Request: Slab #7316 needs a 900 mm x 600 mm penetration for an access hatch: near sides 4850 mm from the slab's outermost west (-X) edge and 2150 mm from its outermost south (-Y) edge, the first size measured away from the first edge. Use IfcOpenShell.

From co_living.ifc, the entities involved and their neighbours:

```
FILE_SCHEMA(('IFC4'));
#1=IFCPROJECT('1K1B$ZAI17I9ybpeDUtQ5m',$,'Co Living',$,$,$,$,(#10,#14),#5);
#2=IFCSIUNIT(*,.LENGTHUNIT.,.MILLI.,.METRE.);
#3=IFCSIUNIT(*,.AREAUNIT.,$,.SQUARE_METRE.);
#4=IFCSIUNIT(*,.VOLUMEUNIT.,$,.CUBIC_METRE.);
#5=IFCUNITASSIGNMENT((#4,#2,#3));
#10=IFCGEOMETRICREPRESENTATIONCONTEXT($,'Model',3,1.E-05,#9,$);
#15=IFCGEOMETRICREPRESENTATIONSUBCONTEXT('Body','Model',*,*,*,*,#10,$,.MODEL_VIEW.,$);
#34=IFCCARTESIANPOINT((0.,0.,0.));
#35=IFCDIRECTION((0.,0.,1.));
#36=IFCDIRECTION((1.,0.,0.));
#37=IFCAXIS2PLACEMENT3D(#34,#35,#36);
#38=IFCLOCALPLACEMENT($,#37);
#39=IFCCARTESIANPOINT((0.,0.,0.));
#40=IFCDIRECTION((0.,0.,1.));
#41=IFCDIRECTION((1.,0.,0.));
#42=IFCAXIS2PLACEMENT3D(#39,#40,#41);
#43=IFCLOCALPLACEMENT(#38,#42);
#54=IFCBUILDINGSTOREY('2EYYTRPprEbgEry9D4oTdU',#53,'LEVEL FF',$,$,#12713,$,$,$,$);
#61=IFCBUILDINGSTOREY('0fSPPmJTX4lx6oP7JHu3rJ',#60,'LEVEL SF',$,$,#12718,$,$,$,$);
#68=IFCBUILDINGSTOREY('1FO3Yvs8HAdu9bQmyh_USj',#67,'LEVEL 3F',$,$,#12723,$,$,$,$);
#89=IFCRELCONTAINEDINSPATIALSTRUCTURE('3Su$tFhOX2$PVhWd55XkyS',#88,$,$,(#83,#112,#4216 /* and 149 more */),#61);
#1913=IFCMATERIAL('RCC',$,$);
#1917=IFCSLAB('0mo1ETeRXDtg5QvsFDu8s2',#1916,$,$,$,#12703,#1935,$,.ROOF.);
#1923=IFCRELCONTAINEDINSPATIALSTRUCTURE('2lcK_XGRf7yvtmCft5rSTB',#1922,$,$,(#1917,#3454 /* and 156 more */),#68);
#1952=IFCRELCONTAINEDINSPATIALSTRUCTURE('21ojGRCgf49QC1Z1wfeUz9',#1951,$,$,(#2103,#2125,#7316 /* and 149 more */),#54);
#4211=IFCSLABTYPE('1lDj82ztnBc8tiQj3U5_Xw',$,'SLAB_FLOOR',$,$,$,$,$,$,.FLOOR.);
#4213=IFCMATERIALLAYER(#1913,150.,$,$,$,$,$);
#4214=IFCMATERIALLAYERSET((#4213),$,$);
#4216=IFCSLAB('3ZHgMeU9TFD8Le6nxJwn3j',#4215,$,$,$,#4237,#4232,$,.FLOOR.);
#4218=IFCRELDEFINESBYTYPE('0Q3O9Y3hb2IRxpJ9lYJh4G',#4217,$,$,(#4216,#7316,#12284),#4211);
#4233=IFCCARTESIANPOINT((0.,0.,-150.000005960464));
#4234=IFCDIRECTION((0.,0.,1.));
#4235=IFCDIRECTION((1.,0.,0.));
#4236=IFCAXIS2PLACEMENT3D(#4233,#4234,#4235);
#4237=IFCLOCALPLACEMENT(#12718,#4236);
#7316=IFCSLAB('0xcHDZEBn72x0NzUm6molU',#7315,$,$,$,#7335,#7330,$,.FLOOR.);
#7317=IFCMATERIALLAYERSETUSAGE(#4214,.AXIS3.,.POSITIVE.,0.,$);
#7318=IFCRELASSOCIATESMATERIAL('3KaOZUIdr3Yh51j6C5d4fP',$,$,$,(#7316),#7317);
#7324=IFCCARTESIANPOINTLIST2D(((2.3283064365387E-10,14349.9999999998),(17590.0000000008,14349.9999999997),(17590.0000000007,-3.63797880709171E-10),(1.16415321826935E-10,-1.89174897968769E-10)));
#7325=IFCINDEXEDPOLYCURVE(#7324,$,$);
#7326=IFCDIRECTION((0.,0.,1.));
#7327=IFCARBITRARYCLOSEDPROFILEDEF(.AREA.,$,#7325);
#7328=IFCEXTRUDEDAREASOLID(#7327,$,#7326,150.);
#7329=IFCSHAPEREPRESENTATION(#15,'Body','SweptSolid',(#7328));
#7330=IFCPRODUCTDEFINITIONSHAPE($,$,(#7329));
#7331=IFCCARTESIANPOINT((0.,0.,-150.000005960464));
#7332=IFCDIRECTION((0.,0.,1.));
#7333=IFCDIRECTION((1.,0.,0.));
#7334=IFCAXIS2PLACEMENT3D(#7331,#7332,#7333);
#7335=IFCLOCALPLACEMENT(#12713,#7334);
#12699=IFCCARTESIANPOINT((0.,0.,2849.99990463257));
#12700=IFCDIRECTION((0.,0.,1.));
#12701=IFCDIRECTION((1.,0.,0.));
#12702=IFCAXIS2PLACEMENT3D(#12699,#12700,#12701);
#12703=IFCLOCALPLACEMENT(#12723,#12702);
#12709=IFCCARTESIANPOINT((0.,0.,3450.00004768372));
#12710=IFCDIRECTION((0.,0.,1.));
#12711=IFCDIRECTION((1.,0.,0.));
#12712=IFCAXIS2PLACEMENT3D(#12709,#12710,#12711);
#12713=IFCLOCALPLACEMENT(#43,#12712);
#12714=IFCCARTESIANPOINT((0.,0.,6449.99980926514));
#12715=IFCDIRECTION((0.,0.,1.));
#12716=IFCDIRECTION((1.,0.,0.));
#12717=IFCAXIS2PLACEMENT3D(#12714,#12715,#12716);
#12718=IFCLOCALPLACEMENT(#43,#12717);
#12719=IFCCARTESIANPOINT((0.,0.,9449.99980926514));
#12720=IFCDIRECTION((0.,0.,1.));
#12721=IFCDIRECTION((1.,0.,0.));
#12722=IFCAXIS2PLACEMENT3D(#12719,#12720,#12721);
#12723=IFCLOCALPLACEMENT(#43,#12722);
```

```python
import numpy as np
import ifcopenshell
import ifcopenshell.api.feature
import ifcopenshell.api.geometry
import ifcopenshell.api.root
import ifcopenshell.geom
import ifcopenshell.util.placement
import ifcopenshell.util.representation
import ifcopenshell.util.shape
import ifcopenshell.util.unit

model = ifcopenshell.open("co_living.ifc")
unit_scale = ifcopenshell.util.unit.calculate_unit_scale(model)
settings = ifcopenshell.geom.settings()


def volume(element):
    """Net volume in cubic metres, openings subtracted."""
    shape = ifcopenshell.geom.create_shape(settings, element)
    return ifcopenshell.util.shape.get_volume(shape.geometry)


slab = model.by_id(7316)
before = volume(slab)

# Extent in the slab's own axes, in metres. The edges named are its -X and -Y sides.
slab_shape = ifcopenshell.geom.create_shape(settings, slab)
vertices = ifcopenshell.util.shape.get_vertices(slab_shape.geometry)
x_min, y_min, bottom = vertices.min(axis=0)
top = vertices[:, 2].max()

opening = ifcopenshell.api.root.create_entity(model, ifc_class="IfcOpeningElement", name="Access hatch opening", predefined_type="OPENING")
context = ifcopenshell.util.representation.get_context(model, "Model", "Body", "MODEL_VIEW")
width, depth = 0.9, 0.6
outline = [(0.0, 0.0), (width, 0.0), (width, depth), (0.0, depth), (0.0, 0.0)]
# Overshoot both faces by 50 mm so the cut is clean.
shape = ifcopenshell.api.geometry.add_slab_representation(
    model, context=context, depth=top - bottom + 0.1, polyline=outline
)
ifcopenshell.api.geometry.assign_representation(model, product=opening, representation=shape)

matrix = ifcopenshell.util.placement.get_local_placement(slab.ObjectPlacement)
matrix[:, 3] = matrix @ np.append(np.array([x_min + 4.85, y_min + 2.15, bottom - 0.05]) / unit_scale, 1.0)
ifcopenshell.api.geometry.edit_object_placement(model, product=opening, matrix=matrix, is_si=False)
ifcopenshell.api.feature.add_feature(model, feature=opening, element=slab)

after = volume(slab)

print(f"slab volume {before:.3f} -> {after:.3f} m3")

model.write("co_living-out.ifc")
```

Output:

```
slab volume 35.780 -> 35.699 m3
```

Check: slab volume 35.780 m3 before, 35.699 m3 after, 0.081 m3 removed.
